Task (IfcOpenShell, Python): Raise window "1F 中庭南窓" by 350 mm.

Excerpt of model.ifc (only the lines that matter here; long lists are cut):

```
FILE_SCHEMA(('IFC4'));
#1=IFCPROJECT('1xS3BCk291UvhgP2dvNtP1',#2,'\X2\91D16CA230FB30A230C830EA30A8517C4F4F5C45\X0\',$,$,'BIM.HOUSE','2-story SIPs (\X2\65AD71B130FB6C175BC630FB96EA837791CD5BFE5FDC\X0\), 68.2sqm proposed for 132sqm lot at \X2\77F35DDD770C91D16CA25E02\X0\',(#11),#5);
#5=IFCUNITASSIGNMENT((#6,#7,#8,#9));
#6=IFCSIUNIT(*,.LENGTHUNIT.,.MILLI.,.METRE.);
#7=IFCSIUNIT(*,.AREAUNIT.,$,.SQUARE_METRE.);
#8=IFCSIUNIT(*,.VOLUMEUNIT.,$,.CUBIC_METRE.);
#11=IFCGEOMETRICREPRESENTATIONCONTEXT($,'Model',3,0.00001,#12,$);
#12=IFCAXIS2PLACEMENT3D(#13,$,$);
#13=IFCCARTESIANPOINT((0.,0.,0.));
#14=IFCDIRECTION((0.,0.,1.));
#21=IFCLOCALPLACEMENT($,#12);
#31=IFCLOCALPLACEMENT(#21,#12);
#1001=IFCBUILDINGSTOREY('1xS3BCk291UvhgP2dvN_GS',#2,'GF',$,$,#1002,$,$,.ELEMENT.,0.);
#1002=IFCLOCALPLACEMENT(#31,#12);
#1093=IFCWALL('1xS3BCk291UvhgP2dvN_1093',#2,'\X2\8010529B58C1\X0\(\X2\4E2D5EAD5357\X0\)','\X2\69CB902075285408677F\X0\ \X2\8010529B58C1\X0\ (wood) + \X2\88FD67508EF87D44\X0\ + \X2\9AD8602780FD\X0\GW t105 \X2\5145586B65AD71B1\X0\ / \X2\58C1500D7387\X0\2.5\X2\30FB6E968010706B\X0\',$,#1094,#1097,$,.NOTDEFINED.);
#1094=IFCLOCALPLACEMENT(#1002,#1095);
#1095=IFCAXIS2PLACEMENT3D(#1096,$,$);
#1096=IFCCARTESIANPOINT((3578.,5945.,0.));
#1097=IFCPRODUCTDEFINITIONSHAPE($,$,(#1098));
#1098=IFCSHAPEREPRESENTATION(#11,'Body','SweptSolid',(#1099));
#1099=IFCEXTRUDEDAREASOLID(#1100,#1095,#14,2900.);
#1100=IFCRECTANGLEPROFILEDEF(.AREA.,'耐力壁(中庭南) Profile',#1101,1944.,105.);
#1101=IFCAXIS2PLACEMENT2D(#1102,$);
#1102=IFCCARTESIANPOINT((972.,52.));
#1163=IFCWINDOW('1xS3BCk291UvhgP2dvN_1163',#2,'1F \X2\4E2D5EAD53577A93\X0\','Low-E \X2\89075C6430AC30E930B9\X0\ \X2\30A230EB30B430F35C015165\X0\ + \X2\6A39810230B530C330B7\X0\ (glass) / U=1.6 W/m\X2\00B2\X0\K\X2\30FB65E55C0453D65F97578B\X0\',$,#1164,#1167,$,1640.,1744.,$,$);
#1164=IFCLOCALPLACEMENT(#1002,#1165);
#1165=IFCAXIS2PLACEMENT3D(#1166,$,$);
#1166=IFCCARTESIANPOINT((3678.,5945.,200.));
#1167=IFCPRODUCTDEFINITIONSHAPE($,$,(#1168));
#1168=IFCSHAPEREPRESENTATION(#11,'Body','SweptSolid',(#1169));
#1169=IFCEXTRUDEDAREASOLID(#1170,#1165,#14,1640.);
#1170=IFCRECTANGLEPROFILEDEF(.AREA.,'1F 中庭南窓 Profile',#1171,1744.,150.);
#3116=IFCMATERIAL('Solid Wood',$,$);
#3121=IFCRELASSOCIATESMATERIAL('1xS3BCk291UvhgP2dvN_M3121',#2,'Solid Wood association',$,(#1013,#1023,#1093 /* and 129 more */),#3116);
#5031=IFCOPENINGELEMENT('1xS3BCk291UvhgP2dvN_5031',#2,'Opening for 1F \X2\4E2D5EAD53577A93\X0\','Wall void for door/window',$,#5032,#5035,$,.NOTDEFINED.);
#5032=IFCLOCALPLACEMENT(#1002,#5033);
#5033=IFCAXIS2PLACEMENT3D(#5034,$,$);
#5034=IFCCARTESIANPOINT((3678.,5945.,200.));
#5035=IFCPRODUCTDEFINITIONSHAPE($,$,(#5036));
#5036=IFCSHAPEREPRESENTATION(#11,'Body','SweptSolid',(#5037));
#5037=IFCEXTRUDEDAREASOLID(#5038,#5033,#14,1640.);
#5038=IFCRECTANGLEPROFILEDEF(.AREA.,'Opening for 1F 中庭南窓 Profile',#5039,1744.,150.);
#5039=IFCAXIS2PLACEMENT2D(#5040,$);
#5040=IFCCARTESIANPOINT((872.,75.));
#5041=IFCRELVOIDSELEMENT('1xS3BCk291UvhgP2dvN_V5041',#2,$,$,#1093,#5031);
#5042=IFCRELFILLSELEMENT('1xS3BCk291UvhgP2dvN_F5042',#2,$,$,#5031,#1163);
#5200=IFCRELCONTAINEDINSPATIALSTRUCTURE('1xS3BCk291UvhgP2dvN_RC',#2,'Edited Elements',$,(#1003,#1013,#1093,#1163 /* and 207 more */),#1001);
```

```python
import numpy as np
import ifcopenshell
import ifcopenshell.api.geometry
import ifcopenshell.util.placement
import ifcopenshell.util.unit

model = ifcopenshell.open("model.ifc")
unit_scale = ifcopenshell.util.unit.calculate_unit_scale(model)

window = model.by_id(1163)
opening = window.FillsVoids[0].RelatingOpeningElement
dz = 0.35 / unit_scale

shift = np.array([0.0, 0.0, dz])
# The window is not placed relative to its opening, so move both.
for product in (opening, window):
    matrix = ifcopenshell.util.placement.get_local_placement(product.ObjectPlacement)
    matrix[:3, 3] += shift
    ifcopenshell.api.geometry.edit_object_placement(model, product=product, matrix=matrix, is_si=False)

print(f"moved by {dz * unit_scale:+.3f} m")

model.write("model_edited.ifc")
```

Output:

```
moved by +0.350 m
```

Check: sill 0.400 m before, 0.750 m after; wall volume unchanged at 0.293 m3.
